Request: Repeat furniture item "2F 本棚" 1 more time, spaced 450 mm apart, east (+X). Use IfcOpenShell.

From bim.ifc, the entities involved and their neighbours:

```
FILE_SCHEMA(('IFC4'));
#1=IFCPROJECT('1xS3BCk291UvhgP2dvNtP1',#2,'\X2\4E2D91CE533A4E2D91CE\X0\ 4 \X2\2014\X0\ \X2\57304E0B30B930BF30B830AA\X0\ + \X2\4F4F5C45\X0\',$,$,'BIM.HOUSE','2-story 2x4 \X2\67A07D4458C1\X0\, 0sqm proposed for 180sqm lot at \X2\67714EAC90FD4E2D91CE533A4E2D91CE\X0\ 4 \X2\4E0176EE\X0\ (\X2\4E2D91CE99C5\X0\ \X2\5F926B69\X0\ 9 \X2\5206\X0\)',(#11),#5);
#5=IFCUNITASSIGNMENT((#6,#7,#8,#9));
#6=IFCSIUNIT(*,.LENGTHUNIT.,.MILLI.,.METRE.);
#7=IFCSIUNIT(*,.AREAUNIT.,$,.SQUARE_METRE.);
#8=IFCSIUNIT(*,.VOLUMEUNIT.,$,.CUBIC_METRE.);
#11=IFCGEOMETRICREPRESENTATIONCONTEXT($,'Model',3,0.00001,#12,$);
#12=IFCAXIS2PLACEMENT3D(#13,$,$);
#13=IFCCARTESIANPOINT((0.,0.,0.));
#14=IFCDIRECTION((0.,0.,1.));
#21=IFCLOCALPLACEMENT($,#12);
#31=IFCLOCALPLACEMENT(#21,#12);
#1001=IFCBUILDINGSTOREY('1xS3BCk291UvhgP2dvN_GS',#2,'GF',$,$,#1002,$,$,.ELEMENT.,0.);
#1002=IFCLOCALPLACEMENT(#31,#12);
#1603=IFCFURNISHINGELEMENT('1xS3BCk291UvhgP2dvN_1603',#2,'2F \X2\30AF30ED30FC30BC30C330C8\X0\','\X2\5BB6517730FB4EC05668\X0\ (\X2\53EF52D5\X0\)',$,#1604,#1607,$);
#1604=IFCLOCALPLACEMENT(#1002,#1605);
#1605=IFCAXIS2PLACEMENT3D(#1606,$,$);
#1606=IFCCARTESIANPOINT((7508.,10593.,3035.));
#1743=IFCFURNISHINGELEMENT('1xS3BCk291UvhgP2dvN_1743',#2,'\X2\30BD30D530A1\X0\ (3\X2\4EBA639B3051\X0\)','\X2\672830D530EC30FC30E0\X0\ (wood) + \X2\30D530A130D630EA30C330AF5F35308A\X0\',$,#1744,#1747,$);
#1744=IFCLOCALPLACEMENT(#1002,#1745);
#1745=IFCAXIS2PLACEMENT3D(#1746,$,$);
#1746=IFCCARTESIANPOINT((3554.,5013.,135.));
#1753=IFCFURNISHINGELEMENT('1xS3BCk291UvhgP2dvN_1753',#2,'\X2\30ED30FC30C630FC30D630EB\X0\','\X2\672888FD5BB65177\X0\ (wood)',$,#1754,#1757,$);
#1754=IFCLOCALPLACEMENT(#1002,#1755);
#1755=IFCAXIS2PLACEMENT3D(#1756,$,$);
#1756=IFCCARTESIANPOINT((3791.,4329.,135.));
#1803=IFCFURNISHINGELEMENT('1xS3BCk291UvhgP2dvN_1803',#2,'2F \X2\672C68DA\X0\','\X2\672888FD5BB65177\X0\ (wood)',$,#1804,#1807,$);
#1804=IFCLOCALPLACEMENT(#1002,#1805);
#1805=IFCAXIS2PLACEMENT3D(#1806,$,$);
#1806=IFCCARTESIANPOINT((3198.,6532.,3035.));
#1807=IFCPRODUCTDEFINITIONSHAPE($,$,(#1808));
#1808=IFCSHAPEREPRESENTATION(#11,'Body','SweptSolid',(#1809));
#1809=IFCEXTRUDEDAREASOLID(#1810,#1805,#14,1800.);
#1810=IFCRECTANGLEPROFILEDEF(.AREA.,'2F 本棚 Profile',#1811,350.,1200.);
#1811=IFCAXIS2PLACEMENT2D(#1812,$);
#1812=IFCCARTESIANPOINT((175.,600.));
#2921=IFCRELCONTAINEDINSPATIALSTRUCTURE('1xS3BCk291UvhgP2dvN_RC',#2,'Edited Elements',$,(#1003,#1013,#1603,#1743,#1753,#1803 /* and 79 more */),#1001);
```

```python
import numpy as np
import ifcopenshell
import ifcopenshell.api.geometry
import ifcopenshell.api.root
import ifcopenshell.util.element
import ifcopenshell.util.placement

model = ifcopenshell.open("bim.ifc")


def reuse_history(source, copy):
    """copy_class also copies each property set's owner history, people and application; keep the originals."""
    for rel in copy.IsDefinedBy:
        if rel.is_a("IfcRelDefinesByProperties") and (history := rel.RelatingPropertyDefinition.OwnerHistory):
            rel.RelatingPropertyDefinition.OwnerHistory = source.OwnerHistory
            ifcopenshell.util.element.remove_deep2(model, history)


source = model.by_guid("1xS3BCk291UvhgP2dvN_1803")
base = ifcopenshell.util.placement.get_local_placement(source.ObjectPlacement)
step = np.array([1.0, 0.0, 0.0]) * 450.0

for i in range(1, 2):
    copy = ifcopenshell.api.root.copy_class(model, product=source)
    copy.Representation = ifcopenshell.util.element.copy_deep(
        model, source.Representation, exclude=["IfcGeometricRepresentationContext", "IfcRepresentationMap"]
    )
    reuse_history(source, copy)
    matrix = base.copy()
    matrix[:3, 3] += i * step
    print("added at", matrix[:3, 3].round(3) + 0.0)
    ifcopenshell.api.geometry.edit_object_placement(model, product=copy, matrix=matrix, is_si=False)

model.write("bim_updated.ifc")
```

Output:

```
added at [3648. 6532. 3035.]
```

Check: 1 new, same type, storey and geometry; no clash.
